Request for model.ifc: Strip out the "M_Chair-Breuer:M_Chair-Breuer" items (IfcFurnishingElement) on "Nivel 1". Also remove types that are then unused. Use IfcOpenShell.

First a look at what the model holds.

```python
import ifcopenshell
import ifcopenshell.util.element

model = ifcopenshell.open("model.ifc")
print(model.schema)
storey = next(s for s in model.by_type("IfcBuildingStorey") if s.Name == "Nivel 1")
furniture = [e for e in ifcopenshell.util.element.get_decomposition(storey) if e.is_a("IfcFurnishingElement")]
seen = {}
for e in furniture:
    element_type = ifcopenshell.util.element.get_type(e)
    name = element_type.Name if element_type not in (None, e) else None
    seen[name] = seen.get(name, 0) + 1
for name, count in sorted(seen.items(), key=str):
    print(count, "x", name)
```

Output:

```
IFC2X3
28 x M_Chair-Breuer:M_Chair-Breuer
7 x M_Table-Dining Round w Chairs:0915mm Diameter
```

```python
import ifcopenshell
import ifcopenshell.api.root
import ifcopenshell.util.element

model = ifcopenshell.open("model.ifc")

storey = next(s for s in model.by_type("IfcBuildingStorey") if s.Name == "Nivel 1")
furniture = [e for e in ifcopenshell.util.element.get_decomposition(storey) if e.is_a("IfcFurnishingElement")]
targets = [e for e in furniture if (t := ifcopenshell.util.element.get_type(e)) not in (None, e) and t.Name == "M_Chair-Breuer:M_Chair-Breuer"]
types = {ifcopenshell.util.element.get_type(e) for e in targets} - {None, *targets}

for e in targets:
    ifcopenshell.api.root.remove_product(model, product=e)
print(len(targets), "removed")

unused = [t for t in types if not ifcopenshell.util.element.get_types(t)]
for t in unused:
    ifcopenshell.api.root.remove_product(model, product=t)
print(len(unused), "unused types removed")

model.write("model-out.ifc")
```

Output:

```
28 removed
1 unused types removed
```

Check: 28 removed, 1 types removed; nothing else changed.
